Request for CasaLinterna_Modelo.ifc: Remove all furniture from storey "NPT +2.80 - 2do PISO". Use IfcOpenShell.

First a look at what the model holds.

```python
import ifcopenshell
import ifcopenshell.util.element

model = ifcopenshell.open("CasaLinterna_Modelo.ifc")
print(model.schema)
storey = next(s for s in model.by_type("IfcBuildingStorey") if s.Name == "NPT +2.80 - 2do PISO")
furniture = [e for e in ifcopenshell.util.element.get_decomposition(storey) if e.is_a("IfcFurnishingElement")]
seen = {}
for e in furniture:
    element_type = ifcopenshell.util.element.get_type(e)
    name = element_type.Name if element_type not in (None, e) else None
    seen[name] = seen.get(name, 0) + 1
for name, count in sorted(seen.items(), key=str):
    print(count, "x", name)
```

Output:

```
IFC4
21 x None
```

```python
import ifcopenshell
import ifcopenshell.api.root
import ifcopenshell.util.element

model = ifcopenshell.open("CasaLinterna_Modelo.ifc")

storey = next(s for s in model.by_type("IfcBuildingStorey") if s.Name == "NPT +2.80 - 2do PISO")
furniture = [e for e in ifcopenshell.util.element.get_decomposition(storey) if e.is_a("IfcFurnishingElement")]

for e in furniture:
    ifcopenshell.api.root.remove_product(model, product=e)
print(len(furniture), "removed")

model.write("CasaLinterna_Modelo_updated.ifc")
```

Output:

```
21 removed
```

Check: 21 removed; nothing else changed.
